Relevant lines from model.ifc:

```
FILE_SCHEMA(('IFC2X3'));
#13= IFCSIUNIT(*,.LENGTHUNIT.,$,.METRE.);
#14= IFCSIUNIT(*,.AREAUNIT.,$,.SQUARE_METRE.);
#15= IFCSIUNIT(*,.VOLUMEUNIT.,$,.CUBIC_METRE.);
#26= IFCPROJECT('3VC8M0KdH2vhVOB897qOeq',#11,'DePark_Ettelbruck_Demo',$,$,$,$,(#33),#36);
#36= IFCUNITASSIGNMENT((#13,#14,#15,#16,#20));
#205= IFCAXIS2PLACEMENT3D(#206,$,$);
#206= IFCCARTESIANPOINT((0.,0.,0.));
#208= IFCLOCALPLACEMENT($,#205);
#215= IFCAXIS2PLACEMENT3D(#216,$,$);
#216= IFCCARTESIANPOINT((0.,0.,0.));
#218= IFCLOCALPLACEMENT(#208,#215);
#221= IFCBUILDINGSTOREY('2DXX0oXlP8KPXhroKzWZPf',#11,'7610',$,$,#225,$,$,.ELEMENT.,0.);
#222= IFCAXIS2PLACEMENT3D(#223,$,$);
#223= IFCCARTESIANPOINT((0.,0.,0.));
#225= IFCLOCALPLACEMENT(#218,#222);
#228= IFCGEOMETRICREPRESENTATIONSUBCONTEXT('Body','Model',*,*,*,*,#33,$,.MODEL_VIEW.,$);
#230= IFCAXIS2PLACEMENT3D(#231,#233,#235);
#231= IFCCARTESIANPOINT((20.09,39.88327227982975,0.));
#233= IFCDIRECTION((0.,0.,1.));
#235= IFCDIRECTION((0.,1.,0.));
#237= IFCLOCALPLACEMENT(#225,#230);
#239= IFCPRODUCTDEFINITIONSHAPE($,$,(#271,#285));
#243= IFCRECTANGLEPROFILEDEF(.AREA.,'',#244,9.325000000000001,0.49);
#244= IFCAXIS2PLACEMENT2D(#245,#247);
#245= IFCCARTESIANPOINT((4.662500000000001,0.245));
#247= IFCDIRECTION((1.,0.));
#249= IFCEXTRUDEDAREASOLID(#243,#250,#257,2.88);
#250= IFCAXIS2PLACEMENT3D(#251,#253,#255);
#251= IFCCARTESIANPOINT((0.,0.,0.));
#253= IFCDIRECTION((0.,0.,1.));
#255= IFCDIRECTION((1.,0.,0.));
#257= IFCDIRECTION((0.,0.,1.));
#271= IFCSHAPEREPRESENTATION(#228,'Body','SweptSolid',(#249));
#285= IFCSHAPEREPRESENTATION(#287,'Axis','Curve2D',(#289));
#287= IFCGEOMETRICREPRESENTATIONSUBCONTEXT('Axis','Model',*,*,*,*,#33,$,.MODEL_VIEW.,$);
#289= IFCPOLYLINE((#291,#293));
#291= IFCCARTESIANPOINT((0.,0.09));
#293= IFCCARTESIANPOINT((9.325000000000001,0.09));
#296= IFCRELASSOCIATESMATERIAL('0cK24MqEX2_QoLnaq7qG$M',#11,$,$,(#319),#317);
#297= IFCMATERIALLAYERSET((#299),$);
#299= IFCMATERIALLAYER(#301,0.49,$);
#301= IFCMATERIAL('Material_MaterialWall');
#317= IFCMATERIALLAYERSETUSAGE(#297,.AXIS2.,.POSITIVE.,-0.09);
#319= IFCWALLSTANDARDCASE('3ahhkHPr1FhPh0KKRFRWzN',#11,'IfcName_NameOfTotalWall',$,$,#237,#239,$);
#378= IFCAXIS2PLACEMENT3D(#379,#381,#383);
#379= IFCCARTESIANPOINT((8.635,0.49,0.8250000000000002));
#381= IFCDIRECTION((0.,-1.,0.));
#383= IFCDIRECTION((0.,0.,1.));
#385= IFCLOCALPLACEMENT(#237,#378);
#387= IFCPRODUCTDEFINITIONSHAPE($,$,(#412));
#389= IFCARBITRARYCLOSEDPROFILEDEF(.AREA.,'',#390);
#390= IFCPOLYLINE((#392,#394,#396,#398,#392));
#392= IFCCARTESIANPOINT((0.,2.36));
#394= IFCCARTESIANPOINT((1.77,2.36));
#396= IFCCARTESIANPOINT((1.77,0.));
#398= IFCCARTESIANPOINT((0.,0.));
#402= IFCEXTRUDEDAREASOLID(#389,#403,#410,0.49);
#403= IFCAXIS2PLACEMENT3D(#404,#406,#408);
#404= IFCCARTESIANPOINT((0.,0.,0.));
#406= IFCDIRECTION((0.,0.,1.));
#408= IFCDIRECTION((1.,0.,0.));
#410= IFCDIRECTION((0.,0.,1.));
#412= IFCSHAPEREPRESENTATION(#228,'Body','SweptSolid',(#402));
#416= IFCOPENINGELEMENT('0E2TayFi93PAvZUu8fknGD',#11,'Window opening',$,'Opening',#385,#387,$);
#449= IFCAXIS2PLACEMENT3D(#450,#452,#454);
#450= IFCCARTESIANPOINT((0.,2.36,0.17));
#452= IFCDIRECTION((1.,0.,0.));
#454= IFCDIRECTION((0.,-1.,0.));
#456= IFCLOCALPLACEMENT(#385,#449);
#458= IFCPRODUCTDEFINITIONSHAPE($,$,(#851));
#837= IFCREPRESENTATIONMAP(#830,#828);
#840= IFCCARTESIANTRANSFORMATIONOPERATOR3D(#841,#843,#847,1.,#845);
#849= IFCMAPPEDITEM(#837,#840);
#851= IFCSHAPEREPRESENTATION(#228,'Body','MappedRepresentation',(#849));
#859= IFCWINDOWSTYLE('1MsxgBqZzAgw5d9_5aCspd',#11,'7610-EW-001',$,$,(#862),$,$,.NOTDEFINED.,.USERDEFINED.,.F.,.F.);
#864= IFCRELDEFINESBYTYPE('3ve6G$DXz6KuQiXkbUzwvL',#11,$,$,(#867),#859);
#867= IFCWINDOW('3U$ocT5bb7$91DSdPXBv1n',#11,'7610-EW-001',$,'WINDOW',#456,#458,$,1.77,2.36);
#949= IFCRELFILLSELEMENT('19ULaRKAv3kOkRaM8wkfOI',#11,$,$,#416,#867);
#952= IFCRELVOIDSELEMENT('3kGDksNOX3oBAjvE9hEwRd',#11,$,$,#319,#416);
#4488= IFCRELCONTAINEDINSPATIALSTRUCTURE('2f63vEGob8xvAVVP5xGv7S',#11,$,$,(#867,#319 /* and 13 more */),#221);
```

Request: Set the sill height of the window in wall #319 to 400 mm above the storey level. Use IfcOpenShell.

```python
import numpy as np
import ifcopenshell
import ifcopenshell.api.geometry
import ifcopenshell.geom
import ifcopenshell.util.element
import ifcopenshell.util.placement
import ifcopenshell.util.shape
import ifcopenshell.util.unit

model = ifcopenshell.open("model.ifc")
unit_scale = ifcopenshell.util.unit.calculate_unit_scale(model)

window = model.by_guid("3U$ocT5bb7$91DSdPXBv1n")
opening = window.FillsVoids[0].RelatingOpeningElement
storey = ifcopenshell.util.element.get_container(window, ifc_class="IfcBuildingStorey")
level = ifcopenshell.util.placement.get_local_placement(storey.ObjectPlacement)[2, 3]

# The opening's origin need not be at the sill, so measure its lowest point.
shape = ifcopenshell.geom.create_shape(ifcopenshell.geom.settings(), opening)
bottom = ifcopenshell.util.shape.get_shape_bottom_elevation(shape, shape.geometry) / unit_scale
dz = level + 0.4 / unit_scale - bottom

shift = np.array([0.0, 0.0, dz])
# The window is placed relative to its opening, so it follows when the opening moves.
matrix = ifcopenshell.util.placement.get_local_placement(opening.ObjectPlacement)
matrix[:3, 3] += shift
ifcopenshell.api.geometry.edit_object_placement(
    model, product=opening, matrix=matrix, is_si=False, should_transform_children=True
)

print(f"moved by {dz * unit_scale:+.3f} m")

model.write("model_rev.ifc")
```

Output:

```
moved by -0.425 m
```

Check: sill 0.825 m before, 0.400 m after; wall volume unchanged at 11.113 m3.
